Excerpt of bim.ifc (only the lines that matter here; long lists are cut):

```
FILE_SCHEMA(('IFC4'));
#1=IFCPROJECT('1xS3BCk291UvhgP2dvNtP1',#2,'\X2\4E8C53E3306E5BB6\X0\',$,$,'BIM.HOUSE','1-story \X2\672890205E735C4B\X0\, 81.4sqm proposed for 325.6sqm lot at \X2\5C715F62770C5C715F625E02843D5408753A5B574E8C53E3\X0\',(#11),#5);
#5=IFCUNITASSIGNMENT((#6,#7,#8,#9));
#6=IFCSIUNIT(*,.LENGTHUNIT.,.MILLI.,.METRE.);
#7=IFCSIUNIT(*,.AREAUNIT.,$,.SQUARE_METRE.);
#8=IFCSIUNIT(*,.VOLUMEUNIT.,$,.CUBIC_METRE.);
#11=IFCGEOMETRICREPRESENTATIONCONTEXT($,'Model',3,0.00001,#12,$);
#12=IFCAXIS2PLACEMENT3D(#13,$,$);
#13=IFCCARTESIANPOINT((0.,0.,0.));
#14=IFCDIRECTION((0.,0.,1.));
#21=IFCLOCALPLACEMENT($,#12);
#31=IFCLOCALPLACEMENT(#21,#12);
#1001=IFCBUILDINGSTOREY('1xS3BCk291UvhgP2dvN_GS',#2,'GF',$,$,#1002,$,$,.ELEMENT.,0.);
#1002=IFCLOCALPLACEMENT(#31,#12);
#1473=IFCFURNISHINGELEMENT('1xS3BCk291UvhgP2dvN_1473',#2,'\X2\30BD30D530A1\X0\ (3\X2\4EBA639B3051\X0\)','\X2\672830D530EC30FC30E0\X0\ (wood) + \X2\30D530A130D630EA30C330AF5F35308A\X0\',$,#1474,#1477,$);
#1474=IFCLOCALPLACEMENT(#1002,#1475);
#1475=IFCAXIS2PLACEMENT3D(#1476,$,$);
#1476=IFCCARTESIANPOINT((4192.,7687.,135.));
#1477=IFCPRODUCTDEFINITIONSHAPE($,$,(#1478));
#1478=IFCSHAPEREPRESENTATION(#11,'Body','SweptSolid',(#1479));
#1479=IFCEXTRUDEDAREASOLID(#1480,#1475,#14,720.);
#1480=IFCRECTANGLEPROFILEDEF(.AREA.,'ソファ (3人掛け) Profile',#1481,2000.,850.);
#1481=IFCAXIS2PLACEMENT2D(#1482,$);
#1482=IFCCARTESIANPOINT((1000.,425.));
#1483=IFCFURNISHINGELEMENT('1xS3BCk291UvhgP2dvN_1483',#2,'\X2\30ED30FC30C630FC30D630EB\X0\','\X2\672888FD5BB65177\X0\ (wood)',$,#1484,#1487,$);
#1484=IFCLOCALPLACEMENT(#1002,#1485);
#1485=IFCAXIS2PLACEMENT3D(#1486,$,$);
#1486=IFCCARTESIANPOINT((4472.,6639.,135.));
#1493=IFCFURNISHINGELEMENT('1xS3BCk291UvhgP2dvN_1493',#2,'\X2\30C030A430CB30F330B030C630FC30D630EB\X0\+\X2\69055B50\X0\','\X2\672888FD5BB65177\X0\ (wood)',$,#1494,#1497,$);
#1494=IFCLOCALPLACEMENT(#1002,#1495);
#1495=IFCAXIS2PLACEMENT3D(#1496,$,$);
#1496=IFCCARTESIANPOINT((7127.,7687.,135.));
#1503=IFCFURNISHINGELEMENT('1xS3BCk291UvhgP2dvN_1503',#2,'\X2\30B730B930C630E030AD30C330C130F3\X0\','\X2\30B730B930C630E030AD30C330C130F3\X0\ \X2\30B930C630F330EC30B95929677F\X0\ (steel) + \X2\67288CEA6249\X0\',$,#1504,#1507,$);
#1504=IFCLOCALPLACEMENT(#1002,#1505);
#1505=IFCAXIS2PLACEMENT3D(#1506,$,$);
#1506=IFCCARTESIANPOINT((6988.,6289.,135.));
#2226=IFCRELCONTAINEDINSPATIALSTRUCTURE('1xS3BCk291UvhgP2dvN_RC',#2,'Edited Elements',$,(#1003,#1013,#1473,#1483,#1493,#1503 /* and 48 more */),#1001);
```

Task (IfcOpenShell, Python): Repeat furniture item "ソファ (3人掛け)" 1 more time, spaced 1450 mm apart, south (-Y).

```python
import numpy as np
import ifcopenshell
import ifcopenshell.api.geometry
import ifcopenshell.api.root
import ifcopenshell.util.element
import ifcopenshell.util.placement

model = ifcopenshell.open("bim.ifc")


def reuse_history(source, copy):
    """copy_class also copies each property set's owner history, people and application; keep the originals."""
    for rel in copy.IsDefinedBy:
        if rel.is_a("IfcRelDefinesByProperties") and (history := rel.RelatingPropertyDefinition.OwnerHistory):
            rel.RelatingPropertyDefinition.OwnerHistory = source.OwnerHistory
            ifcopenshell.util.element.remove_deep2(model, history)


source = model.by_guid("1xS3BCk291UvhgP2dvN_1473")
base = ifcopenshell.util.placement.get_local_placement(source.ObjectPlacement)
step = np.array([0.0, -1.0, 0.0]) * 1450.0

for i in range(1, 2):
    copy = ifcopenshell.api.root.copy_class(model, product=source)
    copy.Representation = ifcopenshell.util.element.copy_deep(
        model, source.Representation, exclude=["IfcGeometricRepresentationContext", "IfcRepresentationMap"]
    )
    reuse_history(source, copy)
    matrix = base.copy()
    matrix[:3, 3] += i * step
    print("added at", matrix[:3, 3].round(3) + 0.0)
    ifcopenshell.api.geometry.edit_object_placement(model, product=copy, matrix=matrix, is_si=False)

model.write("bim-out.ifc")
```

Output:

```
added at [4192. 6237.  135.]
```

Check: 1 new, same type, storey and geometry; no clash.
